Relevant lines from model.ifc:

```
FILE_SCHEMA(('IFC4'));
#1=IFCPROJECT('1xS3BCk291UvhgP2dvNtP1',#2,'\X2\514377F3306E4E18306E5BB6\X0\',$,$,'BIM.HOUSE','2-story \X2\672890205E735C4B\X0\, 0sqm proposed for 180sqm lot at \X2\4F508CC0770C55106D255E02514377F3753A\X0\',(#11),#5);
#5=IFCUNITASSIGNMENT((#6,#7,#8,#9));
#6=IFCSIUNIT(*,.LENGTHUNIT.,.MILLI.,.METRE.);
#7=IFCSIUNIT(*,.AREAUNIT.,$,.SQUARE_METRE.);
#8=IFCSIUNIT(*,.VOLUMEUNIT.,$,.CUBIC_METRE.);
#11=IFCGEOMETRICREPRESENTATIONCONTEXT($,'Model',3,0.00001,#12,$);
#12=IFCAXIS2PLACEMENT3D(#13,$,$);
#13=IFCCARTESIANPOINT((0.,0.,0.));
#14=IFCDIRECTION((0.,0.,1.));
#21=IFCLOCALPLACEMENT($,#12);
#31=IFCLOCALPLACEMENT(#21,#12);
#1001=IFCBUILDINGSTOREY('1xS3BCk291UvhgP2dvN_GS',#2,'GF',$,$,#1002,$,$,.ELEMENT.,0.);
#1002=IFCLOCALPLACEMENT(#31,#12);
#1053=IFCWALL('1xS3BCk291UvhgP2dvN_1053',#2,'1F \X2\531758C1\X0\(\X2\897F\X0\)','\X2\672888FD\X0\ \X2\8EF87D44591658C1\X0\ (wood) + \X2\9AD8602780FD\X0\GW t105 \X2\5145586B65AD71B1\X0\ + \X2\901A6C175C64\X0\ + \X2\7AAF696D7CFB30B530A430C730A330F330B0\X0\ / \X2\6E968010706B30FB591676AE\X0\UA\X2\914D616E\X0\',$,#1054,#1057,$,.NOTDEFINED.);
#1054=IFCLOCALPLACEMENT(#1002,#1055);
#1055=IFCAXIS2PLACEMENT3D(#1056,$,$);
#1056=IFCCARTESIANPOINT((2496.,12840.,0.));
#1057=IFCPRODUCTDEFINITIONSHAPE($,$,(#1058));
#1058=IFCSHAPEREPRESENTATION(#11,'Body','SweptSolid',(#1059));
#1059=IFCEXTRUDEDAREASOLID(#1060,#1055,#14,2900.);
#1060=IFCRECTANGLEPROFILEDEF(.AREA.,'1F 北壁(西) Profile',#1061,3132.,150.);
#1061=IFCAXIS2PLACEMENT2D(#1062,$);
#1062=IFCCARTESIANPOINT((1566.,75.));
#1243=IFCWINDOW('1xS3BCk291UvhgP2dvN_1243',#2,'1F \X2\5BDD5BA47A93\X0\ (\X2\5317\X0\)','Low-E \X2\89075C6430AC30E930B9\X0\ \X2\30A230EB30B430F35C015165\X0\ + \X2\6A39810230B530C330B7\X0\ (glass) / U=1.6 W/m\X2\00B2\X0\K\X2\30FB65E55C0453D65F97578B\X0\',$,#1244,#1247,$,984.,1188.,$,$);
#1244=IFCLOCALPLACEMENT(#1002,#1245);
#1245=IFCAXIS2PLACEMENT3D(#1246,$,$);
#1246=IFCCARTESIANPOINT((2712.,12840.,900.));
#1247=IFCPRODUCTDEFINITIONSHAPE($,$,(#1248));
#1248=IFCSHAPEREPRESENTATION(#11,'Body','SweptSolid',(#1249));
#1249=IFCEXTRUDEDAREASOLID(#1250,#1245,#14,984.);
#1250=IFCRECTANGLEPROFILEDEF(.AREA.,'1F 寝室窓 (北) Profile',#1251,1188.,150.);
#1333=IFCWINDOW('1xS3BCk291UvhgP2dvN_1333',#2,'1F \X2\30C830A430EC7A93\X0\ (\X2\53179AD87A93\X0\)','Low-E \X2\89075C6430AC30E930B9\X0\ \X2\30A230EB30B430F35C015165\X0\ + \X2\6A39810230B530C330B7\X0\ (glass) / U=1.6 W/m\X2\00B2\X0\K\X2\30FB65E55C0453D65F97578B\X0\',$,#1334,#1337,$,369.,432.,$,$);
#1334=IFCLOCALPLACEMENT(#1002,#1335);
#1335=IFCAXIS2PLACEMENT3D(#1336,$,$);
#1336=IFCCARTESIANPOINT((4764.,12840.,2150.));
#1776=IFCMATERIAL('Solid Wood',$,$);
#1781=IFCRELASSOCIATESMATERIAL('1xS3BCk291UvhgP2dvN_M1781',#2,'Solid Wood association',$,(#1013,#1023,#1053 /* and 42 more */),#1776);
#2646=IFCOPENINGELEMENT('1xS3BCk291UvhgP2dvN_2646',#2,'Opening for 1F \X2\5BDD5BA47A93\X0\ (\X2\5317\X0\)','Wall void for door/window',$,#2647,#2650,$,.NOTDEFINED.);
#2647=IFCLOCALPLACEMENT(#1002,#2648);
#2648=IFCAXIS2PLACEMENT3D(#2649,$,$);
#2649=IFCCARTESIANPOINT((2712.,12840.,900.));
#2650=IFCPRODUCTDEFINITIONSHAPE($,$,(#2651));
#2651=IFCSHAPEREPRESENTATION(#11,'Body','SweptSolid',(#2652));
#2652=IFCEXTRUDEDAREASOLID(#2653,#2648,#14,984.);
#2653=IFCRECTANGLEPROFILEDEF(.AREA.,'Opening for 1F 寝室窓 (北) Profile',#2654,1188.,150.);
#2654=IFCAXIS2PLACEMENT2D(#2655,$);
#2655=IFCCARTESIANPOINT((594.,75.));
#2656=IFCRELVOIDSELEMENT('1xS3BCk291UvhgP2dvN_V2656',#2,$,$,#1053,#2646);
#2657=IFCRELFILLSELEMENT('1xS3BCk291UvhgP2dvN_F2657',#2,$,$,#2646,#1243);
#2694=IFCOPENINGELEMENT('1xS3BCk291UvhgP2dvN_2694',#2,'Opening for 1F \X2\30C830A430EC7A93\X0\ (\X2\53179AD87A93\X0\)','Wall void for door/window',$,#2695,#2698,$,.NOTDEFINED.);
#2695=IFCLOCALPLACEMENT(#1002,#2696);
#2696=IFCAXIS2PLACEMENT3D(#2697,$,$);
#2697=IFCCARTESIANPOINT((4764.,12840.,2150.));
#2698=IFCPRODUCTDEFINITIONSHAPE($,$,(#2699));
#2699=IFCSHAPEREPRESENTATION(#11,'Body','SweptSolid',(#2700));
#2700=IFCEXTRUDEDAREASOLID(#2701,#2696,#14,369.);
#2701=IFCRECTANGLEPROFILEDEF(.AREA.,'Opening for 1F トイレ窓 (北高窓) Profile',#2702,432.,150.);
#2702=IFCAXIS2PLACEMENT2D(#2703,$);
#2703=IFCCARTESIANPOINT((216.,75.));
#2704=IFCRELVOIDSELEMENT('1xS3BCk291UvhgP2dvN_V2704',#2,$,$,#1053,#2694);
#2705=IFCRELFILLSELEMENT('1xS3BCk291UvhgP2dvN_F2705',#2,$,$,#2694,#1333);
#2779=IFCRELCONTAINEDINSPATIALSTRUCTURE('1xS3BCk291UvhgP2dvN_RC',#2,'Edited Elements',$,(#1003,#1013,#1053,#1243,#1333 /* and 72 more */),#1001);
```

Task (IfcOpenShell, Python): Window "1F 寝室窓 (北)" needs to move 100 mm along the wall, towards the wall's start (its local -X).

```python
import ifcopenshell
import ifcopenshell.api.geometry
import ifcopenshell.util.placement
import ifcopenshell.util.unit

model = ifcopenshell.open("model.ifc")
unit_scale = ifcopenshell.util.unit.calculate_unit_scale(model)

window = model.by_guid("1xS3BCk291UvhgP2dvN_1243")
opening = window.FillsVoids[0].RelatingOpeningElement
wall = opening.VoidsElements[0].RelatingBuildingElement

wall_matrix = ifcopenshell.util.placement.get_local_placement(wall.ObjectPlacement)
shift = wall_matrix[:3, 0] * -0.1 / unit_scale
before = ifcopenshell.util.placement.get_local_placement(window.ObjectPlacement)[:3, 3].copy()

# The window is not placed relative to its opening, so move both.
for product in (opening, window):
    matrix = ifcopenshell.util.placement.get_local_placement(product.ObjectPlacement)
    matrix[:3, 3] += shift
    ifcopenshell.api.geometry.edit_object_placement(model, product=product, matrix=matrix, is_si=False)

after = ifcopenshell.util.placement.get_local_placement(window.ObjectPlacement)[:3, 3]
print("window moved by", (after - before).round(3) + 0.0)

model.write("model-out.ifc")
```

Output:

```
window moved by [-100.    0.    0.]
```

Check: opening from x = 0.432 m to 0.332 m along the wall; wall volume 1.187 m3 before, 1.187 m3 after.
